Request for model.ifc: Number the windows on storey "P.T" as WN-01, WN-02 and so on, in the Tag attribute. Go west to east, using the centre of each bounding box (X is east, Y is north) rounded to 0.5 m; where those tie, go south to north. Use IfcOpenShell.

First a look at what the model holds.

```python
import ifcopenshell
import ifcopenshell.util.element
import ifcopenshell.util.placement

model = ifcopenshell.open("model.ifc")
print(model.schema)
storey = next(s for s in model.by_type("IfcBuildingStorey") if s.Name == "P.T")
windows = [e for e in ifcopenshell.util.element.get_decomposition(storey) if e.is_a("IfcWindow")]
for e in sorted(windows, key=lambda e: e.id()):
    origin = ifcopenshell.util.placement.get_local_placement(e.ObjectPlacement)[:3, 3]
    print(e.id(), e.Tag, e.Name, origin.round(2) + 0.0, sep=" | ")
```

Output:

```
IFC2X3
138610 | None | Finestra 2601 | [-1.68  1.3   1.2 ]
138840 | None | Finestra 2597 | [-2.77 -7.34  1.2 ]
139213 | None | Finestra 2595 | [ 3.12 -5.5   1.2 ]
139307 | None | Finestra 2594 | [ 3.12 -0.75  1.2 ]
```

```python
import ifcopenshell
import ifcopenshell.geom
import ifcopenshell.util.element
import ifcopenshell.util.shape

model = ifcopenshell.open("model.ifc")
settings = ifcopenshell.geom.settings()
settings.set("use-world-coords", True)


def centre(element):
    shape = ifcopenshell.geom.create_shape(settings, element)
    return ifcopenshell.util.shape.get_bbox_centroid(shape.geometry)


storey = next(s for s in model.by_type("IfcBuildingStorey") if s.Name == "P.T")
windows = [e for e in ifcopenshell.util.element.get_decomposition(storey) if e.is_a("IfcWindow")]

# Insertion points can sit at a corner or the storey origin, so sort by the geometry (in metres).
centres = {e: centre(e) for e in windows}
windows.sort(key=lambda e: (round(centres[e][0] / 0.5), centres[e][1]))

for i, e in enumerate(windows, start=1):
    number = f"WN-{i:02d}"
    e.Tag = number
    print(e.id(), number)

model.write("model_updated.ifc")
```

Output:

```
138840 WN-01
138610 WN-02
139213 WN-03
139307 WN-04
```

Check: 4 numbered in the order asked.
